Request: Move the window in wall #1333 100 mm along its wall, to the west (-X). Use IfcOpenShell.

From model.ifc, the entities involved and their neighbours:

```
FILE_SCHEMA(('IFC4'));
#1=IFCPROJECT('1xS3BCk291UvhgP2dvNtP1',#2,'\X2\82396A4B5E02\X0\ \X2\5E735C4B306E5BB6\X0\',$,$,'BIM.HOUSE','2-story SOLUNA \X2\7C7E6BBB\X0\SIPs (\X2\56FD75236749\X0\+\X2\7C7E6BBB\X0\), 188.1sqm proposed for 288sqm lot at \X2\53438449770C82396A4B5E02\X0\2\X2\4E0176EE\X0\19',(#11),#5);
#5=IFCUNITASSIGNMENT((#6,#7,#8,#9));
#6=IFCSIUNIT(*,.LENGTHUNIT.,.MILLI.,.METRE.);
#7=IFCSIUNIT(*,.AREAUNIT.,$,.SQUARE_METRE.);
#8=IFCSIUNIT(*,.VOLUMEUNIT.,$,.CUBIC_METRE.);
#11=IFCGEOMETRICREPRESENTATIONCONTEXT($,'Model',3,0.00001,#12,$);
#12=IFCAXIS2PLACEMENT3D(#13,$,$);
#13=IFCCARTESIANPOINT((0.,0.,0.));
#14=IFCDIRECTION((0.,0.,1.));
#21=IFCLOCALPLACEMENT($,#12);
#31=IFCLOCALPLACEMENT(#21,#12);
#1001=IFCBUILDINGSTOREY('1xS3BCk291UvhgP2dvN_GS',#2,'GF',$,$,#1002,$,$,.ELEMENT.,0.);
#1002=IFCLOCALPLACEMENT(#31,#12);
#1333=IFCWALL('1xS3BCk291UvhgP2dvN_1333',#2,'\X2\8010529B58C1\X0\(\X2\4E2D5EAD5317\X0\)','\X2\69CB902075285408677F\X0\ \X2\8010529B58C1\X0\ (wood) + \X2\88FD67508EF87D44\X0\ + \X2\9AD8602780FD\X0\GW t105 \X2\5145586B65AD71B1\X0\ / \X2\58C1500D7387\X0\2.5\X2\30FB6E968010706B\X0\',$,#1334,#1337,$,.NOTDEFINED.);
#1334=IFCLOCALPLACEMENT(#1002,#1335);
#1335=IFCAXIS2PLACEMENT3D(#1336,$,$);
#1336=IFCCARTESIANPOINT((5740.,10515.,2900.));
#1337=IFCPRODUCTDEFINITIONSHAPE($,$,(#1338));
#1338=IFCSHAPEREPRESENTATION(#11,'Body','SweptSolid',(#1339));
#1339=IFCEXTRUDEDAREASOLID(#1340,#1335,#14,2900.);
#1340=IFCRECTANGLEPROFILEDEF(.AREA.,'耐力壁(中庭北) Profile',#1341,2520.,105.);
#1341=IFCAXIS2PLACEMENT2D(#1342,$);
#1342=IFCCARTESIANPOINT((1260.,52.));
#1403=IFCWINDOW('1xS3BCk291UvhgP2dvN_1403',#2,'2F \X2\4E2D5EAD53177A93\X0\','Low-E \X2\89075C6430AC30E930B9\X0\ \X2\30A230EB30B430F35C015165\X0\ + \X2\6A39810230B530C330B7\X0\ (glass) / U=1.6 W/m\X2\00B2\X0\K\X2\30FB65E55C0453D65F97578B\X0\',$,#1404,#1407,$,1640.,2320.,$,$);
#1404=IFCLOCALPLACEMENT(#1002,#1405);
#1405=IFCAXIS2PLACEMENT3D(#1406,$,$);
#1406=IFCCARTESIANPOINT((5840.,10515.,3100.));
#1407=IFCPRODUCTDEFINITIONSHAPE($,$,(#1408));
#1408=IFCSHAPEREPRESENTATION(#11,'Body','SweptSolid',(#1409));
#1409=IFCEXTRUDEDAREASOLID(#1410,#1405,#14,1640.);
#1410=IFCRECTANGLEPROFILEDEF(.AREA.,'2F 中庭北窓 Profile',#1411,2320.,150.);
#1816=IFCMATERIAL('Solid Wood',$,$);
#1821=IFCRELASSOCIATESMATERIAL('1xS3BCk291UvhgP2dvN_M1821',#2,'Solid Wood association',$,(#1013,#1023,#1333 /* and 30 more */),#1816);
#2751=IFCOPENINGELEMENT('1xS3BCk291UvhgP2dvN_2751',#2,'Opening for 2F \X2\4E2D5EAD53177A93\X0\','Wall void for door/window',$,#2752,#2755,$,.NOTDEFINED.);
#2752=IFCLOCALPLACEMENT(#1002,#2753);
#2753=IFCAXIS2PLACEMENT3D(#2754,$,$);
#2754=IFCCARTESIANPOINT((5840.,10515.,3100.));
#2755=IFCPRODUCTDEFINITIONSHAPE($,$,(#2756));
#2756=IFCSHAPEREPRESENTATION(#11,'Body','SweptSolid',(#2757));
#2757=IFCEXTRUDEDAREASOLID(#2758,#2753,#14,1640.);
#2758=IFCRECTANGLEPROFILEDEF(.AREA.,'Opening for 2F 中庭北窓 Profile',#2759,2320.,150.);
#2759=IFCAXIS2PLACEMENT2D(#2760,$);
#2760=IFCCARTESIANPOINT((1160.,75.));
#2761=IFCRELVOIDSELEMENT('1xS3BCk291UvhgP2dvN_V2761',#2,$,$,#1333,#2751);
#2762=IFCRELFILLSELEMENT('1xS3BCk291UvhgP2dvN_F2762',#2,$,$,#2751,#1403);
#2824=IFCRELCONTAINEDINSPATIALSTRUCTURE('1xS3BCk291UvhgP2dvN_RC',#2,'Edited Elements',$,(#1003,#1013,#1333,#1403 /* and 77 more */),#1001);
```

```python
import ifcopenshell
import ifcopenshell.api.geometry
import ifcopenshell.util.placement

model = ifcopenshell.open("model.ifc")

window = model.by_guid("1xS3BCk291UvhgP2dvN_1403")
opening = window.FillsVoids[0].RelatingOpeningElement
wall = opening.VoidsElements[0].RelatingBuildingElement

wall_matrix = ifcopenshell.util.placement.get_local_placement(wall.ObjectPlacement)
shift = wall_matrix[:3, 0] * -100.0
before = ifcopenshell.util.placement.get_local_placement(window.ObjectPlacement)[:3, 3].copy()

# The window is not placed relative to its opening, so move both.
for product in (opening, window):
    matrix = ifcopenshell.util.placement.get_local_placement(product.ObjectPlacement)
    matrix[:3, 3] += shift
    ifcopenshell.api.geometry.edit_object_placement(model, product=product, matrix=matrix, is_si=False)

after = ifcopenshell.util.placement.get_local_placement(window.ObjectPlacement)[:3, 3]
print("window moved by", (after - before).round(3) + 0.0)

model.write("model_edited.ifc")
```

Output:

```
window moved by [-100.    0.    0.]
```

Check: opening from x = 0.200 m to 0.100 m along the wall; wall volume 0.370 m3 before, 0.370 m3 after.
